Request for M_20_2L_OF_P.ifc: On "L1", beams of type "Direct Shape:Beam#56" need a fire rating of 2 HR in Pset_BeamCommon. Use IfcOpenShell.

First a look at what the model holds.

```python
import ifcopenshell
import ifcopenshell.util.element

model = ifcopenshell.open("M_20_2L_OF_P.ifc")
print(model.schema)
storey = next(s for s in model.by_type("IfcBuildingStorey") if s.Name == "L1")
beams = [e for e in ifcopenshell.util.element.get_decomposition(storey) if e.is_a("IfcBeam")]
seen = {}
for e in beams:
    element_type = ifcopenshell.util.element.get_type(e)
    key = (element_type.Name if element_type != e and element_type else None, ifcopenshell.util.element.get_pset(e, "Pset_BeamCommon", "FireRating"))
    seen[key] = seen.get(key, 0) + 1
for (name, value), count in sorted(seen.items(), key=str):
    print(count, "x", name, "|", value)
```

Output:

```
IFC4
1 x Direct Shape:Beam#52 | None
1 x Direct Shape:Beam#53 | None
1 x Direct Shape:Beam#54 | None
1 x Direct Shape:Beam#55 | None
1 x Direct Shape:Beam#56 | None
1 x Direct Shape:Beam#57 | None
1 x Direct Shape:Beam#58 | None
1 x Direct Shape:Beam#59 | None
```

```python
import ifcopenshell
import ifcopenshell.api.pset
import ifcopenshell.util.element

model = ifcopenshell.open("M_20_2L_OF_P.ifc")

storey = next(s for s in model.by_type("IfcBuildingStorey") if s.Name == "L1")
beams = [e for e in ifcopenshell.util.element.get_decomposition(storey) if e.is_a("IfcBeam")]

count = 0
for e in beams:
    element_type = ifcopenshell.util.element.get_type(e)
    if element_type in (None, e) or element_type.Name != "Direct Shape:Beam#56":
        continue
    # add_pset returns the element's existing set when there is one.
    pset = ifcopenshell.api.pset.add_pset(model, product=e, name="Pset_BeamCommon")
    ifcopenshell.api.pset.edit_pset(model, pset=pset, properties={"FireRating": "2 HR"})
    count += 1

print(count, "beams updated")

model.write("M_20_2L_OF_P_edited.ifc")
```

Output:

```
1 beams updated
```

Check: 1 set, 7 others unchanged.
